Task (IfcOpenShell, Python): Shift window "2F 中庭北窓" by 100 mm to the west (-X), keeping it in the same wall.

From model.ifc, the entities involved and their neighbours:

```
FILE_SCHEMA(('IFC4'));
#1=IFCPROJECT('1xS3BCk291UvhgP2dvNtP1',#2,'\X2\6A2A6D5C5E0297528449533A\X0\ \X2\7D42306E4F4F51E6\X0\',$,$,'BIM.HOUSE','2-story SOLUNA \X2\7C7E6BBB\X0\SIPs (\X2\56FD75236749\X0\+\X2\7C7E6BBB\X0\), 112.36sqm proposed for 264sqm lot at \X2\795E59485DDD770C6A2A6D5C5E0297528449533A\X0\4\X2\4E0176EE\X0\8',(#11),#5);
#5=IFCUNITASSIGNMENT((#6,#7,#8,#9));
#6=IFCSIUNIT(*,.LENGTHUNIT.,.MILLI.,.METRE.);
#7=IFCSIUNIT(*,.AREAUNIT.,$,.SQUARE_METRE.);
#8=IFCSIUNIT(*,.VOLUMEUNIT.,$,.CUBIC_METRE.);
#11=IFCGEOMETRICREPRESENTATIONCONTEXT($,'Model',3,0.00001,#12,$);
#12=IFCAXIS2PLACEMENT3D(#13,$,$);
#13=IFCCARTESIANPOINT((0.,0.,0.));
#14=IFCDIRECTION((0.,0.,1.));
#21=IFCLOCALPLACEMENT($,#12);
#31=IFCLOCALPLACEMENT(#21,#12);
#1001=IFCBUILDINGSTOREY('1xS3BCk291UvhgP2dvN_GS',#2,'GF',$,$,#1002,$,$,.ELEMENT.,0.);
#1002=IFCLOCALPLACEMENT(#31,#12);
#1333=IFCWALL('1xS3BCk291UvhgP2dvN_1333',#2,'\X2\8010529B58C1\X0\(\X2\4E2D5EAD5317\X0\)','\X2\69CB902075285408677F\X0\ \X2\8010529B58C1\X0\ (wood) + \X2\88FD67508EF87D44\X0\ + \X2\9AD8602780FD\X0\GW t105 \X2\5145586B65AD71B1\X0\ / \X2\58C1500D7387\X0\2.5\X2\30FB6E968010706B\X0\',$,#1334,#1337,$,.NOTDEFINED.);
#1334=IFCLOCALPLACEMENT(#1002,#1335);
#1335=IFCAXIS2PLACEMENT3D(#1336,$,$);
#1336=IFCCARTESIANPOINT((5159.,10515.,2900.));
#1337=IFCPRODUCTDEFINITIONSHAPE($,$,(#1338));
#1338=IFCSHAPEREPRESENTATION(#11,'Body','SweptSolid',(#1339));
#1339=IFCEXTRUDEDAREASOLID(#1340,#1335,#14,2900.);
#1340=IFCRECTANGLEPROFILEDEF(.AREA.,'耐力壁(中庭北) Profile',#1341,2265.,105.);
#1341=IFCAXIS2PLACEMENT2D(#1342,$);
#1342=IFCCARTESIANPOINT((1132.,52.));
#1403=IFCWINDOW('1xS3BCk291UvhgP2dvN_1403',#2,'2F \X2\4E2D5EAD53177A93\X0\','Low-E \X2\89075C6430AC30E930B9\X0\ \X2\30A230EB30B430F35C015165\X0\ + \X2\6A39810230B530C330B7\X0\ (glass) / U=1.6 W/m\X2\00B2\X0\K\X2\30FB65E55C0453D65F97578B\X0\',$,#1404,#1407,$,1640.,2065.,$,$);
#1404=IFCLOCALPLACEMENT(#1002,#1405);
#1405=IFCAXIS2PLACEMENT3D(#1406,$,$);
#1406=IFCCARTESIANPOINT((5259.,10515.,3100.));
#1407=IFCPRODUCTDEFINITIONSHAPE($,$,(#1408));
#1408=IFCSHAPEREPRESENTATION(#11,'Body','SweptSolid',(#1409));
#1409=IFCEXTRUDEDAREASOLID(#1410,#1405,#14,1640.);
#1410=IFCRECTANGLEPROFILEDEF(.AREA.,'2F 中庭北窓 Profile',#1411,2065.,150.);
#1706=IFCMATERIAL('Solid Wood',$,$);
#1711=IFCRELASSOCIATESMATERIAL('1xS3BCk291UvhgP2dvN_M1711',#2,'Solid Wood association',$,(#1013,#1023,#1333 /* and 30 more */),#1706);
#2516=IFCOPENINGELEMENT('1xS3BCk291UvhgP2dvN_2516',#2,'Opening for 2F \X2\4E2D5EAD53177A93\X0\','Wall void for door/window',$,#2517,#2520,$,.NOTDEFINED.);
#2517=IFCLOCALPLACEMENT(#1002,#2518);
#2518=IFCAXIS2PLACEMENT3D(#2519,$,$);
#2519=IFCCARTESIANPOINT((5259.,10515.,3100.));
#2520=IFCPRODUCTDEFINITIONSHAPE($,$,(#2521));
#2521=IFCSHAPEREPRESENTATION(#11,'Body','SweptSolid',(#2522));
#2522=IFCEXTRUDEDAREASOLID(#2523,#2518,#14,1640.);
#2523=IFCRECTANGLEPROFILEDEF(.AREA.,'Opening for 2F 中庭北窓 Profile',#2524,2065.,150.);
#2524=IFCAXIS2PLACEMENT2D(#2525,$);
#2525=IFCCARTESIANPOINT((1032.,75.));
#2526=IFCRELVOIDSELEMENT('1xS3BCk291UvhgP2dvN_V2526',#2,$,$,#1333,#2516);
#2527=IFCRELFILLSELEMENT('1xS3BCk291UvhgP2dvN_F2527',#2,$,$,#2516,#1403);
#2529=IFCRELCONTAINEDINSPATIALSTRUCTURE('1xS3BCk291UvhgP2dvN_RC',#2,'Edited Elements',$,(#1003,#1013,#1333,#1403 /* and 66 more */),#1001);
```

```python
import ifcopenshell
import ifcopenshell.api.geometry
import ifcopenshell.util.placement
import ifcopenshell.util.unit

model = ifcopenshell.open("model.ifc")
unit_scale = ifcopenshell.util.unit.calculate_unit_scale(model)

window = model.by_guid("1xS3BCk291UvhgP2dvN_1403")
opening = window.FillsVoids[0].RelatingOpeningElement
wall = opening.VoidsElements[0].RelatingBuildingElement

wall_matrix = ifcopenshell.util.placement.get_local_placement(wall.ObjectPlacement)
shift = wall_matrix[:3, 0] * -0.1 / unit_scale
before = ifcopenshell.util.placement.get_local_placement(window.ObjectPlacement)[:3, 3].copy()

# The window is not placed relative to its opening, so move both.
for product in (opening, window):
    matrix = ifcopenshell.util.placement.get_local_placement(product.ObjectPlacement)
    matrix[:3, 3] += shift
    ifcopenshell.api.geometry.edit_object_placement(model, product=product, matrix=matrix, is_si=False)

after = ifcopenshell.util.placement.get_local_placement(window.ObjectPlacement)[:3, 3]
print("window moved by", (after - before).round(3) + 0.0)

model.write("model_updated.ifc")
```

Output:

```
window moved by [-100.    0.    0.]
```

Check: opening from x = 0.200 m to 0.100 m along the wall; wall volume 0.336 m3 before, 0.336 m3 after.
